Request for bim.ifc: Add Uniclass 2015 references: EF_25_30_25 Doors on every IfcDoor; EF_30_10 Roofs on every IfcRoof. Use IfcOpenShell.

First a look at what the model holds.

```python
import ifcopenshell

model = ifcopenshell.open("bim.ifc")
print(model.schema)
print("classifications:", [c.Name for c in model.by_type("IfcClassification")])
for ifc_class in ("IfcDoor", "IfcRoof", "IfcStair", "IfcWall", "IfcWindow"):
    print(ifc_class, len(model.by_type(ifc_class)))
```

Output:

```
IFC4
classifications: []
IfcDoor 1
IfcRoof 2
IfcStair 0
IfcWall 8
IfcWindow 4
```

```python
import ifcopenshell
import ifcopenshell.api.classification

model = ifcopenshell.open("bim.ifc")

system = ifcopenshell.api.classification.add_classification(model, classification="Uniclass 2015")

codes = {
    "IfcDoor": ("EF_25_30_25", "Doors"),
    "IfcRoof": ("EF_30_10", "Roofs"),
}
for ifc_class, (code, name) in codes.items():
    products = model.by_type(ifc_class)
    ifcopenshell.api.classification.add_reference(
        model, products=products, classification=system, identification=code, name=name
    )
    print(code, len(products))

model.write("bim-out.ifc")
```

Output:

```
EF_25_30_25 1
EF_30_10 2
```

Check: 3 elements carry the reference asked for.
